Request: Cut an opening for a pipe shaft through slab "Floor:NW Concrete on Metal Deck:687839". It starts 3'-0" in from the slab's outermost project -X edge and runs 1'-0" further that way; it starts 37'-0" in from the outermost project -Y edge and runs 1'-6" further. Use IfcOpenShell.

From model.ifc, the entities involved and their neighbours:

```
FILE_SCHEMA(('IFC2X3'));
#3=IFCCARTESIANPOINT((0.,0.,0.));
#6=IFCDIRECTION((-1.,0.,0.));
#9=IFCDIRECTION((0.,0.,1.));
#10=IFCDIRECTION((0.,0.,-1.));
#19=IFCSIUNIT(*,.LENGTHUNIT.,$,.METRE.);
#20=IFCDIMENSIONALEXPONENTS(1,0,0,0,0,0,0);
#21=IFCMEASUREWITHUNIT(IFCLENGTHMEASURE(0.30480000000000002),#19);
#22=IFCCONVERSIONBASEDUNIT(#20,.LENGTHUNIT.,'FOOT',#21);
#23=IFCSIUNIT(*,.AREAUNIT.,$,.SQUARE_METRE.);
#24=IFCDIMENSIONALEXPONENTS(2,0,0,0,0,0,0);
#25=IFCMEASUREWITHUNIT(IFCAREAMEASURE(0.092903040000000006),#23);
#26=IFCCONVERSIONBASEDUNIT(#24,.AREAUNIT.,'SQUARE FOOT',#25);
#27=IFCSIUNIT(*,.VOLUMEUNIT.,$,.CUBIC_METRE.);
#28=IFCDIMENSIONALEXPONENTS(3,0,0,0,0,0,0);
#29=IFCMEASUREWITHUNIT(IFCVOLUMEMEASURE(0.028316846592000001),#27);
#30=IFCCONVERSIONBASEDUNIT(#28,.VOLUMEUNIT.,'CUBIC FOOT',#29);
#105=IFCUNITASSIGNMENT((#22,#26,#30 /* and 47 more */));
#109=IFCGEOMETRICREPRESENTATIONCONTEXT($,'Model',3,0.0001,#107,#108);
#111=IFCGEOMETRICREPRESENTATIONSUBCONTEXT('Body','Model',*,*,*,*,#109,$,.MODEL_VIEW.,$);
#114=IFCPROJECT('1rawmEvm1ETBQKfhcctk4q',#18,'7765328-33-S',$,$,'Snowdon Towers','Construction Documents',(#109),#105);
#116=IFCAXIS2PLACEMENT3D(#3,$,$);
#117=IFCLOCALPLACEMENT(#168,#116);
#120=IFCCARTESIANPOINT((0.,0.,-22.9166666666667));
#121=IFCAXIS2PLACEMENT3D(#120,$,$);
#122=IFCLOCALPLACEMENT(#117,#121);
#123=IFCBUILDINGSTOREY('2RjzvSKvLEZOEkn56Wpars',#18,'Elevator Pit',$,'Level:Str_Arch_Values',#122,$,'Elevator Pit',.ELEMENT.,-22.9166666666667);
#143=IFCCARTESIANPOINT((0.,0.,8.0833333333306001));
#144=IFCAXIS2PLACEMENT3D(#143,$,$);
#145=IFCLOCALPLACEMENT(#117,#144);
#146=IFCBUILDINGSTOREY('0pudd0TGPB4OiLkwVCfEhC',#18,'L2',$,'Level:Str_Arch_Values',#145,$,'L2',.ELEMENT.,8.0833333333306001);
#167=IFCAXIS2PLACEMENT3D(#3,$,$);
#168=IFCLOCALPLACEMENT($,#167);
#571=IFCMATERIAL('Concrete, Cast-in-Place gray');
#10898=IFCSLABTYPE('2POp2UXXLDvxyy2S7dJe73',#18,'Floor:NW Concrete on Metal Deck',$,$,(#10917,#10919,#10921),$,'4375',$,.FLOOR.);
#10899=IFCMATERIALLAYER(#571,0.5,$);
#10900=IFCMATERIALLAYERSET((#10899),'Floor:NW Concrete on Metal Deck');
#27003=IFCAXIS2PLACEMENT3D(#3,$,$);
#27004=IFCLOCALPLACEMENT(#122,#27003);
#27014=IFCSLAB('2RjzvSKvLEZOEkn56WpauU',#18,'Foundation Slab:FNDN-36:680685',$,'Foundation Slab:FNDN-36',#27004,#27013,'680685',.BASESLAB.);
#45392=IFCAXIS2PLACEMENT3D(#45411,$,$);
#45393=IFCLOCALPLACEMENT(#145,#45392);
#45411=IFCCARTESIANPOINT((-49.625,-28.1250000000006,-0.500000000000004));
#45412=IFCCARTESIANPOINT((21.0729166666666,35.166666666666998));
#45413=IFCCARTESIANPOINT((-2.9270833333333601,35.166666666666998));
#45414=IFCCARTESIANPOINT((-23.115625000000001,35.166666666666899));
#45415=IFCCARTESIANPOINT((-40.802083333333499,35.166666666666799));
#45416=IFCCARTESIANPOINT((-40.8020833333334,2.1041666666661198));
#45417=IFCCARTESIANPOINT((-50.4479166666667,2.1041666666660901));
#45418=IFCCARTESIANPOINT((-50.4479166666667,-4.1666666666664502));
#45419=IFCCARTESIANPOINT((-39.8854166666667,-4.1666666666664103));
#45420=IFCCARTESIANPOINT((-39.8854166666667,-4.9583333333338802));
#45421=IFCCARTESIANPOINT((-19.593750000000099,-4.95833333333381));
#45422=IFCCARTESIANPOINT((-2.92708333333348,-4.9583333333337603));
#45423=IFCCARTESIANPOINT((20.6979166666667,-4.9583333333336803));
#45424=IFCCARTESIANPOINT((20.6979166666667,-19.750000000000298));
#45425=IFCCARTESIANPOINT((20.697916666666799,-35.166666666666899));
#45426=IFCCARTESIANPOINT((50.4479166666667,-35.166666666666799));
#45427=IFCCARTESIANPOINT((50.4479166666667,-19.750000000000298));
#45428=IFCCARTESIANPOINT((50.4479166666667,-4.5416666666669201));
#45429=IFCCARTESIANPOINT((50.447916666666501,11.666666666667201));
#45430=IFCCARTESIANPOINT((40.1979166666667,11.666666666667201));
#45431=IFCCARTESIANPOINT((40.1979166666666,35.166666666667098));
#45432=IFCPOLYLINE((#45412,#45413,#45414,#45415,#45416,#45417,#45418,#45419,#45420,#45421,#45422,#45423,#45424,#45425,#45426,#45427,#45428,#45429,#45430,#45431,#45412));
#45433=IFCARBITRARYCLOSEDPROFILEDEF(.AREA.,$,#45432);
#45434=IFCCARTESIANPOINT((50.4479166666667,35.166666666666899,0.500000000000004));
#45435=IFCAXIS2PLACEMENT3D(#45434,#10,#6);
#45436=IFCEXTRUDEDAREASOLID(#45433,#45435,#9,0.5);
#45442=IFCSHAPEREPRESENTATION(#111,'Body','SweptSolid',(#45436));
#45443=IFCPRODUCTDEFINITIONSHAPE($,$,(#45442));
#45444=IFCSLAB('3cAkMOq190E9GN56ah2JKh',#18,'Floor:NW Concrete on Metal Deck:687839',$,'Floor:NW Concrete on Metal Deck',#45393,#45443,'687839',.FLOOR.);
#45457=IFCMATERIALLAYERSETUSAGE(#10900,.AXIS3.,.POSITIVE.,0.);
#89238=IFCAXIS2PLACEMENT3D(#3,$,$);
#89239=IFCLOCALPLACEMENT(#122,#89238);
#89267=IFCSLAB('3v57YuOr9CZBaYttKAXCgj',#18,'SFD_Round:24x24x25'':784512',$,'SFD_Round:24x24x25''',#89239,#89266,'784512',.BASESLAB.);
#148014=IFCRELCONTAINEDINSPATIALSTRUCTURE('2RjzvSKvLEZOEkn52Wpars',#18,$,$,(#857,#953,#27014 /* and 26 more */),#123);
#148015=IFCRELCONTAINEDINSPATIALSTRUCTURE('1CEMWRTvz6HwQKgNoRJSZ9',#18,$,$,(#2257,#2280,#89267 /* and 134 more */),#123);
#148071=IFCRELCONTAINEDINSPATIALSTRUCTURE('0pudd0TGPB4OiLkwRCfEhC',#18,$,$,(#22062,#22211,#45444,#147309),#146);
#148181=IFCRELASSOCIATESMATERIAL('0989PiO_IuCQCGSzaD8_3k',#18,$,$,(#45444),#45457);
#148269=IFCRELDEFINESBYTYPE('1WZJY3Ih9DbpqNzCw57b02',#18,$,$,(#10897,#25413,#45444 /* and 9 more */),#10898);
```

```python
import numpy as np
import ifcopenshell
import ifcopenshell.api.feature
import ifcopenshell.api.geometry
import ifcopenshell.api.root
import ifcopenshell.geom
import ifcopenshell.util.placement
import ifcopenshell.util.representation
import ifcopenshell.util.shape
import ifcopenshell.util.unit

model = ifcopenshell.open("model.ifc")
unit_scale = ifcopenshell.util.unit.calculate_unit_scale(model)
settings = ifcopenshell.geom.settings()


def volume(element):
    """Net volume in cubic metres, openings subtracted."""
    shape = ifcopenshell.geom.create_shape(settings, element)
    return ifcopenshell.util.shape.get_volume(shape.geometry)


slab = model.by_id(45444)
before = volume(slab)

# Extent in the slab's own axes, in metres. The edges named are its -X and -Y sides.
slab_shape = ifcopenshell.geom.create_shape(settings, slab)
vertices = ifcopenshell.util.shape.get_vertices(slab_shape.geometry)
x_min, y_min, bottom = vertices.min(axis=0)
top = vertices[:, 2].max()

opening = ifcopenshell.api.root.create_entity(model, ifc_class="IfcOpeningElement", name="Pipe shaft opening")
context = ifcopenshell.util.representation.get_context(model, "Model", "Body", "MODEL_VIEW")
width, depth = 0.3048, 0.4572
outline = [(0.0, 0.0), (width, 0.0), (width, depth), (0.0, depth), (0.0, 0.0)]
# Overshoot both faces by 50 mm so the cut is clean.
shape = ifcopenshell.api.geometry.add_slab_representation(
    model, context=context, depth=top - bottom + 0.1, polyline=outline
)
ifcopenshell.api.geometry.assign_representation(model, product=opening, representation=shape)

matrix = ifcopenshell.util.placement.get_local_placement(slab.ObjectPlacement)
matrix[:, 3] = matrix @ np.append(np.array([x_min + 0.9144, y_min + 11.2776, bottom - 0.05]) / unit_scale, 1.0)
ifcopenshell.api.geometry.edit_object_placement(model, product=opening, matrix=matrix, is_si=False)
ifcopenshell.api.feature.add_feature(model, feature=opening, element=slab)

after = volume(slab)

print(f"slab volume {before:.3f} -> {after:.3f} m3")

model.write("model_v2.ifc")
```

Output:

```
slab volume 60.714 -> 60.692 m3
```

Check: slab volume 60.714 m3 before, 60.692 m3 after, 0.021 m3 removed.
